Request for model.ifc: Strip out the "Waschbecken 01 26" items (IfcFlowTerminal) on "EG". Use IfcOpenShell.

First a look at what the model holds.

```python
import ifcopenshell
import ifcopenshell.util.element

model = ifcopenshell.open("model.ifc")
print(model.schema)
storey = next(s for s in model.by_type("IfcBuildingStorey") if s.Name == "EG")
terminals = [e for e in ifcopenshell.util.element.get_decomposition(storey) if e.is_a("IfcFlowTerminal")]
seen = {}
for e in terminals:
    element_type = ifcopenshell.util.element.get_type(e)
    name = element_type.Name if element_type not in (None, e) else None
    seen[name] = seen.get(name, 0) + 1
for name, count in sorted(seen.items(), key=str):
    print(count, "x", name)
```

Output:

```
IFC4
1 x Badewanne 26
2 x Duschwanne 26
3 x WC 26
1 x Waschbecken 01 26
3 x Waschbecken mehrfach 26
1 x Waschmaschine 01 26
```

```python
import ifcopenshell
import ifcopenshell.api.root
import ifcopenshell.util.element

model = ifcopenshell.open("model.ifc")

storey = next(s for s in model.by_type("IfcBuildingStorey") if s.Name == "EG")
terminals = [e for e in ifcopenshell.util.element.get_decomposition(storey) if e.is_a("IfcFlowTerminal")]
targets = [e for e in terminals if (t := ifcopenshell.util.element.get_type(e)) not in (None, e) and t.Name == "Waschbecken 01 26"]

for e in targets:
    ifcopenshell.api.root.remove_product(model, product=e)
print(len(targets), "removed")

model.write("model_v2.ifc")
```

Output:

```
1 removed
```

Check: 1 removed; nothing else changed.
